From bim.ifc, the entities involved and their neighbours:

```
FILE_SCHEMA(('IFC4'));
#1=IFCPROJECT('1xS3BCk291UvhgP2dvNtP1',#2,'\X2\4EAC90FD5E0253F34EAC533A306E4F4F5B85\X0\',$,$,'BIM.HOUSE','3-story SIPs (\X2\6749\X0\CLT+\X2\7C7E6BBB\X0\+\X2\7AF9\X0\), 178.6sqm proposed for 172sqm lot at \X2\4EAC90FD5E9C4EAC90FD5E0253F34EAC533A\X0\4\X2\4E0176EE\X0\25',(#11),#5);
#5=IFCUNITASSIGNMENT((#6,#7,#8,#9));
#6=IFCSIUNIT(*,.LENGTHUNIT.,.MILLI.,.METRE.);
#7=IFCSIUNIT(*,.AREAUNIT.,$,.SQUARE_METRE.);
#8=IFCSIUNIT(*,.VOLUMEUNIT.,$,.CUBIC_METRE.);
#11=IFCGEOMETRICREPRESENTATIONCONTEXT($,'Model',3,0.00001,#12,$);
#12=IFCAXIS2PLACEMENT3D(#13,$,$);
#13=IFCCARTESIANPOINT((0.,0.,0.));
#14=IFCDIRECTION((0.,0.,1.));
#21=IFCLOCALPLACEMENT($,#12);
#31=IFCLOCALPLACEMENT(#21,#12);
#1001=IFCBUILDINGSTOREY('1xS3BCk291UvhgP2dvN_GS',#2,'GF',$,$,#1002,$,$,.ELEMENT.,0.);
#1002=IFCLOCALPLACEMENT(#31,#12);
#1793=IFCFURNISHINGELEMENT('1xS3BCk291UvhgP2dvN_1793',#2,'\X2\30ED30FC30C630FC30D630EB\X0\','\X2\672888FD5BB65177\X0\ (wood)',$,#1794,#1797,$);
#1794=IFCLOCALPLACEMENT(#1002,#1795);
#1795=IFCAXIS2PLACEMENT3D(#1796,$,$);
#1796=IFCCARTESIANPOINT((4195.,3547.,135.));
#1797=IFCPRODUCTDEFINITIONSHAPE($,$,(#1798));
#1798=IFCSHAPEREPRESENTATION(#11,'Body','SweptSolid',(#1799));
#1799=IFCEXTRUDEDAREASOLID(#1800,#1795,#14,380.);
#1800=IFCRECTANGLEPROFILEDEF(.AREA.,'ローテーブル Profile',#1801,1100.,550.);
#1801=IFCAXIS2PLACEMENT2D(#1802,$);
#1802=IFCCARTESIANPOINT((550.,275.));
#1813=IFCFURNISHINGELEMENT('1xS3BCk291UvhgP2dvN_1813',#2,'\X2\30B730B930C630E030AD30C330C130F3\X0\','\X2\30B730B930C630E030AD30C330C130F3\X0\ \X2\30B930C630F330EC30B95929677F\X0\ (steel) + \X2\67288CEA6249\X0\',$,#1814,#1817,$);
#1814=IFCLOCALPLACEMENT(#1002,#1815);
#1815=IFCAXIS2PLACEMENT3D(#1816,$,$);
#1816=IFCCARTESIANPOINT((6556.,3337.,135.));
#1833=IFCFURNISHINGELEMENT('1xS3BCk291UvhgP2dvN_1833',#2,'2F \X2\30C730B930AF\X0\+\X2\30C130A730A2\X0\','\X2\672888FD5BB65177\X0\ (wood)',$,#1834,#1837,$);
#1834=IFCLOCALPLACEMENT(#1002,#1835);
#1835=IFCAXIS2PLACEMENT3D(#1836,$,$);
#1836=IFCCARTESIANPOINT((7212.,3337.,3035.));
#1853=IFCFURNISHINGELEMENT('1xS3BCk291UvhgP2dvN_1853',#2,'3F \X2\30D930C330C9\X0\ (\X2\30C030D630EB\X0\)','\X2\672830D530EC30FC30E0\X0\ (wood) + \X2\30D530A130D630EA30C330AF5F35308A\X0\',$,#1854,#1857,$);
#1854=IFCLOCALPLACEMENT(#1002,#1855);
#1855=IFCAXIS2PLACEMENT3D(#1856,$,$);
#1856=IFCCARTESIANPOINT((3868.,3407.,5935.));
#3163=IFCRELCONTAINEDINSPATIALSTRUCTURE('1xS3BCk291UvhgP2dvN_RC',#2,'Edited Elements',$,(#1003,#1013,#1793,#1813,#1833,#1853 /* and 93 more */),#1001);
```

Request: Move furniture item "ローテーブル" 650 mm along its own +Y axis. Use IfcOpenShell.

```python
import ifcopenshell
import ifcopenshell.api.geometry
import ifcopenshell.util.placement
import ifcopenshell.util.unit

model = ifcopenshell.open("bim.ifc")
unit_scale = ifcopenshell.util.unit.calculate_unit_scale(model)

item = model.by_guid("1xS3BCk291UvhgP2dvN_1793")
matrix = ifcopenshell.util.placement.get_local_placement(item.ObjectPlacement)
matrix[:3, 3] += matrix[:3, 1] * 0.65 / unit_scale
ifcopenshell.api.geometry.edit_object_placement(model, product=item, matrix=matrix, is_si=False)

print(ifcopenshell.util.placement.get_local_placement(item.ObjectPlacement).round(3) + 0.0)

model.write("bim_updated.ifc")
```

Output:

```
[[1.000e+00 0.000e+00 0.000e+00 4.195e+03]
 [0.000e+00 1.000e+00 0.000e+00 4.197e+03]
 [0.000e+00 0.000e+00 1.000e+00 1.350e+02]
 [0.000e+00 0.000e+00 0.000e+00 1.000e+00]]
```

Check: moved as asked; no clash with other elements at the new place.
